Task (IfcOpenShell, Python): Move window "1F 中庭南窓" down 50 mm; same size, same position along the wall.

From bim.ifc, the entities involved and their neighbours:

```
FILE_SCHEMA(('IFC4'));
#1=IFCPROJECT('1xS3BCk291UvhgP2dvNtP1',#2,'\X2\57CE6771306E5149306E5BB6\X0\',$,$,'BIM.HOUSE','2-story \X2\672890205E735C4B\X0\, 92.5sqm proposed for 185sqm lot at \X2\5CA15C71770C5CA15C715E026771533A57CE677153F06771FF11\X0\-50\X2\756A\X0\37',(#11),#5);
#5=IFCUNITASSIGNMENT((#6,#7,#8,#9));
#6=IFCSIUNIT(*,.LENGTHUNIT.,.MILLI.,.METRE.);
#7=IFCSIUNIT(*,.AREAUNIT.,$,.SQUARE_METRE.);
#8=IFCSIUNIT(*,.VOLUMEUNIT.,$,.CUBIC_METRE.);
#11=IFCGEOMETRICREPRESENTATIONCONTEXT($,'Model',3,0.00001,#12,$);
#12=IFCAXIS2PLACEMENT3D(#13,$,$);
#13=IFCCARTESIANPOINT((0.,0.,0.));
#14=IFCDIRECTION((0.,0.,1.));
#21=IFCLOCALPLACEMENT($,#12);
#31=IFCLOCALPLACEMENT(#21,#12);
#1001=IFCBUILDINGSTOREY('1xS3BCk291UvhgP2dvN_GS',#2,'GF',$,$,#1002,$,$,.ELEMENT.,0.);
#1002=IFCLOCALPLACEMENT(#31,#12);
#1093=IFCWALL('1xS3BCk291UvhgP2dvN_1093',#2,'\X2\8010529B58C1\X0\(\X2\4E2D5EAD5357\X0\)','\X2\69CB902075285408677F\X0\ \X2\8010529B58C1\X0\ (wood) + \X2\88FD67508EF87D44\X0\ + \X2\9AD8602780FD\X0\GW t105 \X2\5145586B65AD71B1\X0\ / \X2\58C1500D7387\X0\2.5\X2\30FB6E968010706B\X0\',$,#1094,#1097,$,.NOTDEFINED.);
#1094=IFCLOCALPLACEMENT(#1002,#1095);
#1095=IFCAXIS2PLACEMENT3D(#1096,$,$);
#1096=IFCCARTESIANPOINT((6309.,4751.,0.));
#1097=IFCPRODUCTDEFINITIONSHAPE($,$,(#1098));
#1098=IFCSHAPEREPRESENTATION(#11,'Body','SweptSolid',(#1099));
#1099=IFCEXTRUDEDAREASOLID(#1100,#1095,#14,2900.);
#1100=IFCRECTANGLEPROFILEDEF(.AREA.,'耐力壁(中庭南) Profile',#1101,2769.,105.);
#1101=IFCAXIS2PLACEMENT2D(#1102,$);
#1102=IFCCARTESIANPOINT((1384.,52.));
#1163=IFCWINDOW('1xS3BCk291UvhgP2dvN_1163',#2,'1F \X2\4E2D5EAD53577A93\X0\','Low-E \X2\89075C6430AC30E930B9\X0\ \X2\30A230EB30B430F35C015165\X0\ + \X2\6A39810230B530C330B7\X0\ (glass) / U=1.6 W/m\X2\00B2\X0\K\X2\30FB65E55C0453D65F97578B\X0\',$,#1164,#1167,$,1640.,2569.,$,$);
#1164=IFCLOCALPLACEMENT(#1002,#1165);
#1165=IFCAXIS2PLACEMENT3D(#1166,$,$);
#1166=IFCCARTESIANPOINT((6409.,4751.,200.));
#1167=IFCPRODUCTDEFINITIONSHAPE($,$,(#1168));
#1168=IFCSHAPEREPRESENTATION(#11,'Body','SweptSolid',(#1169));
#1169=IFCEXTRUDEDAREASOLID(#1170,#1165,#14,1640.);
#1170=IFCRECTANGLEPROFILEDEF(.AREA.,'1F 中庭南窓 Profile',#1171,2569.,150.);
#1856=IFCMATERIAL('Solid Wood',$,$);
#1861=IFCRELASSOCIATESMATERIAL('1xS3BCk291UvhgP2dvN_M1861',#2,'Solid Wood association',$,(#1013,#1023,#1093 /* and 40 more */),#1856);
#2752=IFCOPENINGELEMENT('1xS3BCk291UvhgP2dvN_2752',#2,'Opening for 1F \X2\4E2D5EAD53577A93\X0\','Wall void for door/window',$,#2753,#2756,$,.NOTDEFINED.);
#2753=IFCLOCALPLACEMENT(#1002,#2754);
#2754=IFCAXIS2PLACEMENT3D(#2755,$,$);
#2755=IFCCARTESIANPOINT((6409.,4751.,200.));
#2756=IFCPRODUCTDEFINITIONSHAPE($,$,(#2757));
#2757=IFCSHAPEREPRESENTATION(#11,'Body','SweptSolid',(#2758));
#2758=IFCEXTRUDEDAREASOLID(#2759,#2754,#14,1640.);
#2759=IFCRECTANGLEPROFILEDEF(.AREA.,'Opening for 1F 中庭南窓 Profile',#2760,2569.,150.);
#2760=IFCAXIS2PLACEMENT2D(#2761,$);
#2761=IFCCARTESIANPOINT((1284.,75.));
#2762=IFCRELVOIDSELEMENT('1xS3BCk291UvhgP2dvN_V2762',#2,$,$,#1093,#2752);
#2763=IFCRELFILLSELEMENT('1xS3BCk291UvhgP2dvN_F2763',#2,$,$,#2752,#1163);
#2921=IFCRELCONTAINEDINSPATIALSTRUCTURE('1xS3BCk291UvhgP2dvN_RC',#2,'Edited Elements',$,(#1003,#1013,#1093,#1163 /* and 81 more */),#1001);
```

```python
import numpy as np
import ifcopenshell
import ifcopenshell.api.geometry
import ifcopenshell.util.placement
import ifcopenshell.util.unit

model = ifcopenshell.open("bim.ifc")
unit_scale = ifcopenshell.util.unit.calculate_unit_scale(model)

window = model.by_guid("1xS3BCk291UvhgP2dvN_1163")
opening = window.FillsVoids[0].RelatingOpeningElement
dz = -50.0

shift = np.array([0.0, 0.0, dz])
# The window is not placed relative to its opening, so move both.
for product in (opening, window):
    matrix = ifcopenshell.util.placement.get_local_placement(product.ObjectPlacement)
    matrix[:3, 3] += shift
    ifcopenshell.api.geometry.edit_object_placement(model, product=product, matrix=matrix, is_si=False)

print(f"moved by {dz * unit_scale:+.3f} m")

model.write("bim_edited.ifc")
```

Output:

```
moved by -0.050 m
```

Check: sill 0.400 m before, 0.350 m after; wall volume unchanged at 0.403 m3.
